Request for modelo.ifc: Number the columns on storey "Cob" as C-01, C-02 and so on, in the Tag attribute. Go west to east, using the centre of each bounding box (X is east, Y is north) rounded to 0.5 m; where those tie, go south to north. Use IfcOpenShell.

First a look at what the model holds.

```python
import ifcopenshell
import ifcopenshell.util.element
import ifcopenshell.util.placement

model = ifcopenshell.open("modelo.ifc")
print(model.schema)
storey = next(s for s in model.by_type("IfcBuildingStorey") if s.Name == "Cob")
columns = [e for e in ifcopenshell.util.element.get_decomposition(storey) if e.is_a("IfcColumn")]
for e in sorted(columns, key=lambda e: e.id()):
    origin = ifcopenshell.util.placement.get_local_placement(e.ObjectPlacement)[:3, 3]
    print(e.id(), e.Tag, e.Name, origin.round(2) + 0.0, sep=" | ")
```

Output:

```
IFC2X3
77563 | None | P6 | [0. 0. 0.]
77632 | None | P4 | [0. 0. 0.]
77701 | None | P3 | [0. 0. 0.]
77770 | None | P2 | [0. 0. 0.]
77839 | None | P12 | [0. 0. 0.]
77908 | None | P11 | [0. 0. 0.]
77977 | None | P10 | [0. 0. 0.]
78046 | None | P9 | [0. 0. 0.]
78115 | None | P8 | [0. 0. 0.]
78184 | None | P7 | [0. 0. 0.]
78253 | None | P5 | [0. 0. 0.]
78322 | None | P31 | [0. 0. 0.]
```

```python
import ifcopenshell
import ifcopenshell.geom
import ifcopenshell.util.element
import ifcopenshell.util.shape

model = ifcopenshell.open("modelo.ifc")
settings = ifcopenshell.geom.settings()
settings.set("use-world-coords", True)


def centre(element):
    shape = ifcopenshell.geom.create_shape(settings, element)
    return ifcopenshell.util.shape.get_bbox_centroid(shape.geometry)


storey = next(s for s in model.by_type("IfcBuildingStorey") if s.Name == "Cob")
columns = [e for e in ifcopenshell.util.element.get_decomposition(storey) if e.is_a("IfcColumn")]

# Insertion points can sit at a corner or the storey origin, so sort by the geometry (in metres).
centres = {e: centre(e) for e in columns}
columns.sort(key=lambda e: (round(centres[e][0] / 0.5), centres[e][1]))

for i, e in enumerate(columns, start=1):
    number = f"C-{i:02d}"
    e.Tag = number
    print(e.id(), number)

model.write("modelo_edited.ifc")
```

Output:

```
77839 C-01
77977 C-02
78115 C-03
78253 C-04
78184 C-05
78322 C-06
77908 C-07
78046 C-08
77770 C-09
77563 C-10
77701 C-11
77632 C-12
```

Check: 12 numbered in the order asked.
